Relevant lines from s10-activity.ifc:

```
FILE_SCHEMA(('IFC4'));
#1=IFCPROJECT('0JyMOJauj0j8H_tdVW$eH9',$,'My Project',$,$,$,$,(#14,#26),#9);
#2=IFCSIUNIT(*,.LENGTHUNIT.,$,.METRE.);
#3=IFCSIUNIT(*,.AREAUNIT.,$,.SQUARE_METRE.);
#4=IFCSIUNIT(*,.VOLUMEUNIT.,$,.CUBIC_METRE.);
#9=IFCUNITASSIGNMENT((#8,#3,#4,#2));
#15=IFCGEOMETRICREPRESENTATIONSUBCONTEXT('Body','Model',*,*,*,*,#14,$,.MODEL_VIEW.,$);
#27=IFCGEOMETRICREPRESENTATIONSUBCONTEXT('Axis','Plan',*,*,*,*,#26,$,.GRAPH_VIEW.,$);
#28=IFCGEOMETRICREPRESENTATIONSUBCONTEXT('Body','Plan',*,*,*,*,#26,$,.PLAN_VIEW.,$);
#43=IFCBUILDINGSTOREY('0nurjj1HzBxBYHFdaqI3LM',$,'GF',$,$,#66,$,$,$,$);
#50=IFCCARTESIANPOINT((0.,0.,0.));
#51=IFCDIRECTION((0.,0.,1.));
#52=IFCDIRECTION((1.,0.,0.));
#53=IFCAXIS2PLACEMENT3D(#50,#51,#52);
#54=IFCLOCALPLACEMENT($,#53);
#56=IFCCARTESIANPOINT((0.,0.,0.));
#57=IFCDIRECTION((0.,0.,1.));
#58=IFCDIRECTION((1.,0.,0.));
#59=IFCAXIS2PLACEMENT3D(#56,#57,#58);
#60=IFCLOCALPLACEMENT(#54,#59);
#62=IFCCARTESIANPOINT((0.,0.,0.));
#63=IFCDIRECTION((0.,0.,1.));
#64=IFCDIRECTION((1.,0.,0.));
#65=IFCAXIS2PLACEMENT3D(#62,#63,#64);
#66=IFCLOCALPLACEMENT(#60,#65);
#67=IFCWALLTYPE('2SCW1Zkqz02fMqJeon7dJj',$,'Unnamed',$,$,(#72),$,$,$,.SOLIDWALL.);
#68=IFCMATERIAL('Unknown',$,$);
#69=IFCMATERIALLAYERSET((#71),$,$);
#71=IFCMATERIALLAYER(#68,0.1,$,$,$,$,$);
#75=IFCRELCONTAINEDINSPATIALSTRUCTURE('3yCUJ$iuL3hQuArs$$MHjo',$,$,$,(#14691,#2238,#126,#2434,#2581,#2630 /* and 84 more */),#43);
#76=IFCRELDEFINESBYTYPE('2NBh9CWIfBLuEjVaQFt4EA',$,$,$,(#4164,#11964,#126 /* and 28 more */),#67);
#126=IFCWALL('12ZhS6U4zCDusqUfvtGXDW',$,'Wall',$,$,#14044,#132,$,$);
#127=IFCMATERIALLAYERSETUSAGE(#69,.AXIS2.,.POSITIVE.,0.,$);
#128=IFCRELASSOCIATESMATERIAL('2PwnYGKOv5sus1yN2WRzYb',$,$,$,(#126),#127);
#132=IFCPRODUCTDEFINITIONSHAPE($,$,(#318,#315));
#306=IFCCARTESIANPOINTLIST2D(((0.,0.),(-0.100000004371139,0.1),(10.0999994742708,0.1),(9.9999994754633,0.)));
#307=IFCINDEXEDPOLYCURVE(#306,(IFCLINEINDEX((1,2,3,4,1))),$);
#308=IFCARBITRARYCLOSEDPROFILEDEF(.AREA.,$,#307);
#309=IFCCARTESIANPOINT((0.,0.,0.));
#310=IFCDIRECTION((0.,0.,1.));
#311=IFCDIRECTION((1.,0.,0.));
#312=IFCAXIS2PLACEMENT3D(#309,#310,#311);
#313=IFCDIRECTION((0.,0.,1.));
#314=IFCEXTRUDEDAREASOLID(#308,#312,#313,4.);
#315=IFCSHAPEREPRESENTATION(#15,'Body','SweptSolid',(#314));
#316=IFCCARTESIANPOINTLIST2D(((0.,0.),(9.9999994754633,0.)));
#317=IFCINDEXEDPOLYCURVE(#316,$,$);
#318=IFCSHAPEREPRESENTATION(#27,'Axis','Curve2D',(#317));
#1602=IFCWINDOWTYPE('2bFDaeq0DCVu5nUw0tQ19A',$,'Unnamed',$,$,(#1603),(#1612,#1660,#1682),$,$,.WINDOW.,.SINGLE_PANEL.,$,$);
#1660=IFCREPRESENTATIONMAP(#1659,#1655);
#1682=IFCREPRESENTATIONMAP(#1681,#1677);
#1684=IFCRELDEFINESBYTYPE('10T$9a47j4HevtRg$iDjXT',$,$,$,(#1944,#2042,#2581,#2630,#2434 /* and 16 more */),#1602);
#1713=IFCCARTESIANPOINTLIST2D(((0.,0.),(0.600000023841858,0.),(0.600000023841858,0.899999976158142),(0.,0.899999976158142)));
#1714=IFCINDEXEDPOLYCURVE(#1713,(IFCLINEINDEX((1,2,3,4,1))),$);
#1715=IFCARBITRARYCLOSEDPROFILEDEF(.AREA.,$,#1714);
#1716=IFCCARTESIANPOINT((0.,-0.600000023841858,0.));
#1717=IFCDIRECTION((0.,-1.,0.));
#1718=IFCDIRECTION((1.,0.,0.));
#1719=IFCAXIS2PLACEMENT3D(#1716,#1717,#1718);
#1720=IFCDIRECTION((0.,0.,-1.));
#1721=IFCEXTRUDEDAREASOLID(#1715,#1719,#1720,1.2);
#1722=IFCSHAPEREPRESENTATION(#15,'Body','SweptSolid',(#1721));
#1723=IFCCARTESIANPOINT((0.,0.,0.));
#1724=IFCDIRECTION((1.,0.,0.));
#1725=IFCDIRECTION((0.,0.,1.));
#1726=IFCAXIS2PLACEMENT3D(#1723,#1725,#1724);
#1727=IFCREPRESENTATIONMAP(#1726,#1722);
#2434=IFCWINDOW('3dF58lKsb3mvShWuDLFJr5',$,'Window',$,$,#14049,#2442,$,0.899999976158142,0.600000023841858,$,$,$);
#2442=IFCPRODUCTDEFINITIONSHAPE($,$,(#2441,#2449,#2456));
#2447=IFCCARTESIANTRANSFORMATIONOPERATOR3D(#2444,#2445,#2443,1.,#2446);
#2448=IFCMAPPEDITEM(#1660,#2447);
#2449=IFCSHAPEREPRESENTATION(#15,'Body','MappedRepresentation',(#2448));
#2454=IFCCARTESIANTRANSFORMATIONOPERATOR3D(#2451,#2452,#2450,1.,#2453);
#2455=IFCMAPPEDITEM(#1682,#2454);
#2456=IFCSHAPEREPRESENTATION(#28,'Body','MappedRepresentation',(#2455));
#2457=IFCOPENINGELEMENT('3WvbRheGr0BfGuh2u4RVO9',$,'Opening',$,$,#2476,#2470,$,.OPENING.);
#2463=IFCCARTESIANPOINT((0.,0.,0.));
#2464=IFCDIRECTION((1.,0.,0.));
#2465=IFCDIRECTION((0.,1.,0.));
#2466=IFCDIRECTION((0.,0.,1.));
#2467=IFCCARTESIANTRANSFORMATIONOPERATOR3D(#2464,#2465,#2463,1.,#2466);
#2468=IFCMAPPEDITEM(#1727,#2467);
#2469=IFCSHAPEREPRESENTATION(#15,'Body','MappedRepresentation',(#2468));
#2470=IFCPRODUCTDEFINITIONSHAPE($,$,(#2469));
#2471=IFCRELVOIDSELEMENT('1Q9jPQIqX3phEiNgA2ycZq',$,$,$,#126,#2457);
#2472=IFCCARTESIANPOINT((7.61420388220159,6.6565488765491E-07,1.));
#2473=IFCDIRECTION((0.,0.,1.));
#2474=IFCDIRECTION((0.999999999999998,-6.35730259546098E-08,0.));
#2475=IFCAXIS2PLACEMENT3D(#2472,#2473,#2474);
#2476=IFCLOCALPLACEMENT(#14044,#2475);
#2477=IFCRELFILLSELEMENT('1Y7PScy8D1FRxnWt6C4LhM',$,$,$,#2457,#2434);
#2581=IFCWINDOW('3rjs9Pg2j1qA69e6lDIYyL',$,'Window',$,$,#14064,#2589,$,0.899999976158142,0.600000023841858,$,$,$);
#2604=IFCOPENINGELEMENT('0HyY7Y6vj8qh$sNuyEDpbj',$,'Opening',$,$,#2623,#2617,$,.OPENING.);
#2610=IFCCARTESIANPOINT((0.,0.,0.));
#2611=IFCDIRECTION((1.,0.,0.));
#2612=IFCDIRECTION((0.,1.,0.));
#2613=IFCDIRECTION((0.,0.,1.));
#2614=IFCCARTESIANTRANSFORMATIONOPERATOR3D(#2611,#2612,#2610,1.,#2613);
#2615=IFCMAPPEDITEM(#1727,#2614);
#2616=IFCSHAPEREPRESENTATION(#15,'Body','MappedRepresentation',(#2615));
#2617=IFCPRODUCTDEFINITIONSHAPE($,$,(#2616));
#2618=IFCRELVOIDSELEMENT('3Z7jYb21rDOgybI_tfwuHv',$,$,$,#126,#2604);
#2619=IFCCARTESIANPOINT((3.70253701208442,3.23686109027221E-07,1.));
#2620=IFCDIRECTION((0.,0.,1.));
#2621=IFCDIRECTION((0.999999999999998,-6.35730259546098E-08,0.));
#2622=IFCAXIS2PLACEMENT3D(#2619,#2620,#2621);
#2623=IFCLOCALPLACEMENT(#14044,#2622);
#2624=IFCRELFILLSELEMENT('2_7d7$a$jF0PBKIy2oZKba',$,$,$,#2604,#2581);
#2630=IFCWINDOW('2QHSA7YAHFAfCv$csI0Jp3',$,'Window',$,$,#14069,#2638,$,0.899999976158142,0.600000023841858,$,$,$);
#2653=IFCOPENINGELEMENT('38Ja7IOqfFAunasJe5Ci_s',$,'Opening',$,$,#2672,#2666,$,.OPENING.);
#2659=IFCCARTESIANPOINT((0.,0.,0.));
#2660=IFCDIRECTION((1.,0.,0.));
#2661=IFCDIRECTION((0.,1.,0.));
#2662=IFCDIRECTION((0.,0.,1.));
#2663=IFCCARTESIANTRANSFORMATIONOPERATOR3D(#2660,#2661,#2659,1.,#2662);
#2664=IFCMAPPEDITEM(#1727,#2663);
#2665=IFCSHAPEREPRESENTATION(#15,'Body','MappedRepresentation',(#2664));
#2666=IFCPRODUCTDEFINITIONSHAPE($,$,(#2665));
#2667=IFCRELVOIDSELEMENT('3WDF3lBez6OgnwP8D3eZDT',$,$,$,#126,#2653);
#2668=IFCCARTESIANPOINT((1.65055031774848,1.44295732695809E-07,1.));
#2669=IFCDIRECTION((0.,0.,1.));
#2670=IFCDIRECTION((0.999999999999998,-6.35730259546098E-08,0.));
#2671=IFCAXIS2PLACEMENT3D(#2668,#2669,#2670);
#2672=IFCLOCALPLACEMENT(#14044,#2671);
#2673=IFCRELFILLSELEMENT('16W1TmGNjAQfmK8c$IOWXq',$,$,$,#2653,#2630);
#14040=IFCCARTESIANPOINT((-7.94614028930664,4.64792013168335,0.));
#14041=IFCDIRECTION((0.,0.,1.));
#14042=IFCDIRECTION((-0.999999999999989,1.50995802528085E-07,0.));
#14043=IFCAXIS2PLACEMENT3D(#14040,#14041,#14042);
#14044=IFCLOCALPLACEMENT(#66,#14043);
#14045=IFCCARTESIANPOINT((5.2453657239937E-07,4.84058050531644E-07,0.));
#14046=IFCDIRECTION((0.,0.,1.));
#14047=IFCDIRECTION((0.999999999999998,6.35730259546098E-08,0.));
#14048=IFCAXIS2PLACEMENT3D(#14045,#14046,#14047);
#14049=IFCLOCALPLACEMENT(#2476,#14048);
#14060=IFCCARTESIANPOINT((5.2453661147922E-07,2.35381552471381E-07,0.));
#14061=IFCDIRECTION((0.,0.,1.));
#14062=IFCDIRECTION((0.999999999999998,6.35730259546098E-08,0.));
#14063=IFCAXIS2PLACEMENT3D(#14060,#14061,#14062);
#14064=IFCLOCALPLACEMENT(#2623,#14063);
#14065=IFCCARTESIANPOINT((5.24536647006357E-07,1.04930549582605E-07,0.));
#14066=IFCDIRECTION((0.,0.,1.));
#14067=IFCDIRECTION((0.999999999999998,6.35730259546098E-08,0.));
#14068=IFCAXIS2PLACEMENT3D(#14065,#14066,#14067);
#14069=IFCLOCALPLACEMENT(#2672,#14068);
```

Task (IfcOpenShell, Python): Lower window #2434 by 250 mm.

```python
import numpy as np
import ifcopenshell
import ifcopenshell.api.geometry
import ifcopenshell.util.placement
import ifcopenshell.util.unit

model = ifcopenshell.open("s10-activity.ifc")
unit_scale = ifcopenshell.util.unit.calculate_unit_scale(model)

window = model.by_guid("3dF58lKsb3mvShWuDLFJr5")
opening = window.FillsVoids[0].RelatingOpeningElement
dz = -0.25 / unit_scale

shift = np.array([0.0, 0.0, dz])
# The window is placed relative to its opening, so it follows when the opening moves.
matrix = ifcopenshell.util.placement.get_local_placement(opening.ObjectPlacement)
matrix[:3, 3] += shift
ifcopenshell.api.geometry.edit_object_placement(
    model, product=opening, matrix=matrix, is_si=False, should_transform_children=True
)

print(f"moved by {dz * unit_scale:+.3f} m")

model.write("s10-activity_v2.ifc")
```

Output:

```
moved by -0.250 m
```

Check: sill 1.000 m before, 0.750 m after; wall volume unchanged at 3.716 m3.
